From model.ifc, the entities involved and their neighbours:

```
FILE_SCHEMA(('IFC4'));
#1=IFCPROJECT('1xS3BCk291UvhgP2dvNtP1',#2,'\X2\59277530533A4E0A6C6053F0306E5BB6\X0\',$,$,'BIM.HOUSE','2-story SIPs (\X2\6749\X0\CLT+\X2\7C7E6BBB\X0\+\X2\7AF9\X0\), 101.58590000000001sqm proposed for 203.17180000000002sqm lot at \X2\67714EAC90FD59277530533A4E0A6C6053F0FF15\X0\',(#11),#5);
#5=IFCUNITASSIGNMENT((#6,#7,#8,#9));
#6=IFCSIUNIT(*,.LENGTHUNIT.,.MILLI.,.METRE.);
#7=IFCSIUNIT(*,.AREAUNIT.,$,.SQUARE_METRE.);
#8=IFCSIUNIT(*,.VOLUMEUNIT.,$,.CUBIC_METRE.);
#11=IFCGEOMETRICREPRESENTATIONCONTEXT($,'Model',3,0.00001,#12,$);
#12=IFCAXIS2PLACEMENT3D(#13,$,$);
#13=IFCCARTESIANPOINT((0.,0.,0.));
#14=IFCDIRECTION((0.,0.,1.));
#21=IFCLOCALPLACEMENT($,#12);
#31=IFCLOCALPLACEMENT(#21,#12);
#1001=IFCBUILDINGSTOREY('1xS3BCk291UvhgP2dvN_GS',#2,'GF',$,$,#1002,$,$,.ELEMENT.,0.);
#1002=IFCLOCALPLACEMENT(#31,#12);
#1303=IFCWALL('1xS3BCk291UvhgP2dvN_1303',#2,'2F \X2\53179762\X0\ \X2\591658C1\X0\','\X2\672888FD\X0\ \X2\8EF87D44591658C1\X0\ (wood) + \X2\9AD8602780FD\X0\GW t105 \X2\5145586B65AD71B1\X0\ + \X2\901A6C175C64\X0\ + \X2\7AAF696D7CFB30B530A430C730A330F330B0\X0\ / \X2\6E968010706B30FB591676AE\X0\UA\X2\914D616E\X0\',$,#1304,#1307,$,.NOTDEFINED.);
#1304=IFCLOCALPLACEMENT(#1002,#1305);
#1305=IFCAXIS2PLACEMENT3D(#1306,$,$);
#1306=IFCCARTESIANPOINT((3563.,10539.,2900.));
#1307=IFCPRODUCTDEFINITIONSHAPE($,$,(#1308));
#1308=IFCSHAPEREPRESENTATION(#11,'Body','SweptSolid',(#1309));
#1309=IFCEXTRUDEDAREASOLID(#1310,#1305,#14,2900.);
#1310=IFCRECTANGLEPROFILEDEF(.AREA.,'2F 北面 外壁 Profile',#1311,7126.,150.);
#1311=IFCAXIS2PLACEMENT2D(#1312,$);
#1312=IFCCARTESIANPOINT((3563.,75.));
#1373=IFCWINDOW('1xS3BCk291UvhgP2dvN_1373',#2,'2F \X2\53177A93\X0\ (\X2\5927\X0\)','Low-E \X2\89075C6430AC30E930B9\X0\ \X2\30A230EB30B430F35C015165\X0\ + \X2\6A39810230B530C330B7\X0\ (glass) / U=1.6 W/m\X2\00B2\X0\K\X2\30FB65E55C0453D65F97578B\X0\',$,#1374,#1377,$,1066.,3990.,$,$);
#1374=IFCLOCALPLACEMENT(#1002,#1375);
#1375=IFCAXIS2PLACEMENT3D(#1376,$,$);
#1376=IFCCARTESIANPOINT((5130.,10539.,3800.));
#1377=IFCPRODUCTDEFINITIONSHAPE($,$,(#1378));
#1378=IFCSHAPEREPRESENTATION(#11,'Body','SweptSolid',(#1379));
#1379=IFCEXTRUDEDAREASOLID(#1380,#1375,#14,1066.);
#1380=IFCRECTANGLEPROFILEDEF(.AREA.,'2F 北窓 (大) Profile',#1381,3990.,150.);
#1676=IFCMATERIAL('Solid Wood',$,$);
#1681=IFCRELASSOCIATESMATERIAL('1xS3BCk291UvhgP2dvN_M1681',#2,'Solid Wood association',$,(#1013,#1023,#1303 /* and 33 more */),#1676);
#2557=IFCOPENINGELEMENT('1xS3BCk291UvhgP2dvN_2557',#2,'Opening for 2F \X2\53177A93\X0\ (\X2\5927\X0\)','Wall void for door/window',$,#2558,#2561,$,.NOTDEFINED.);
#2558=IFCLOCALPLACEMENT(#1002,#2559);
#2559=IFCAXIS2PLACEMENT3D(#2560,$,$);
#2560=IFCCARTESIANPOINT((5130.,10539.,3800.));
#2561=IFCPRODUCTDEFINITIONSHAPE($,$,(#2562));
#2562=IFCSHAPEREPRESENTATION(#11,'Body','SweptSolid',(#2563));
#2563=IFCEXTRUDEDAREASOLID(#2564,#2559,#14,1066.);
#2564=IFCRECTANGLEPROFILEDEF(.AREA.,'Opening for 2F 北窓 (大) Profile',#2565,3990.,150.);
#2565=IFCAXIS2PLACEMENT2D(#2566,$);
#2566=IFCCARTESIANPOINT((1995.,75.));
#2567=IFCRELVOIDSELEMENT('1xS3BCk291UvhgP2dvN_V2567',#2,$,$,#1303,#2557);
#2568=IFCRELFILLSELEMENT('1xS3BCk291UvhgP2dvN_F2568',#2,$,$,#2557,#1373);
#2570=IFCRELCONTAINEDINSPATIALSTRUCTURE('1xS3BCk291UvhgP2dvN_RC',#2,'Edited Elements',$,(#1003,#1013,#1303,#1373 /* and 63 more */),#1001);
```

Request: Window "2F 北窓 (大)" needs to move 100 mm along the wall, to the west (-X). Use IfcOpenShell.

```python
import ifcopenshell
import ifcopenshell.api.geometry
import ifcopenshell.util.placement
import ifcopenshell.util.unit

model = ifcopenshell.open("model.ifc")
unit_scale = ifcopenshell.util.unit.calculate_unit_scale(model)

window = model.by_id(1373)
opening = window.FillsVoids[0].RelatingOpeningElement
wall = opening.VoidsElements[0].RelatingBuildingElement

wall_matrix = ifcopenshell.util.placement.get_local_placement(wall.ObjectPlacement)
shift = wall_matrix[:3, 0] * -0.1 / unit_scale
before = ifcopenshell.util.placement.get_local_placement(window.ObjectPlacement)[:3, 3].copy()

# The window is not placed relative to its opening, so move both.
for product in (opening, window):
    matrix = ifcopenshell.util.placement.get_local_placement(product.ObjectPlacement)
    matrix[:3, 3] += shift
    ifcopenshell.api.geometry.edit_object_placement(model, product=product, matrix=matrix, is_si=False)

after = ifcopenshell.util.placement.get_local_placement(window.ObjectPlacement)[:3, 3]
print("window moved by", (after - before).round(3) + 0.0)

model.write("model-out.ifc")
```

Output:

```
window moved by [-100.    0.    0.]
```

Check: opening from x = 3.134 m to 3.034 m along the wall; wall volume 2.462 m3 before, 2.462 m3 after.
